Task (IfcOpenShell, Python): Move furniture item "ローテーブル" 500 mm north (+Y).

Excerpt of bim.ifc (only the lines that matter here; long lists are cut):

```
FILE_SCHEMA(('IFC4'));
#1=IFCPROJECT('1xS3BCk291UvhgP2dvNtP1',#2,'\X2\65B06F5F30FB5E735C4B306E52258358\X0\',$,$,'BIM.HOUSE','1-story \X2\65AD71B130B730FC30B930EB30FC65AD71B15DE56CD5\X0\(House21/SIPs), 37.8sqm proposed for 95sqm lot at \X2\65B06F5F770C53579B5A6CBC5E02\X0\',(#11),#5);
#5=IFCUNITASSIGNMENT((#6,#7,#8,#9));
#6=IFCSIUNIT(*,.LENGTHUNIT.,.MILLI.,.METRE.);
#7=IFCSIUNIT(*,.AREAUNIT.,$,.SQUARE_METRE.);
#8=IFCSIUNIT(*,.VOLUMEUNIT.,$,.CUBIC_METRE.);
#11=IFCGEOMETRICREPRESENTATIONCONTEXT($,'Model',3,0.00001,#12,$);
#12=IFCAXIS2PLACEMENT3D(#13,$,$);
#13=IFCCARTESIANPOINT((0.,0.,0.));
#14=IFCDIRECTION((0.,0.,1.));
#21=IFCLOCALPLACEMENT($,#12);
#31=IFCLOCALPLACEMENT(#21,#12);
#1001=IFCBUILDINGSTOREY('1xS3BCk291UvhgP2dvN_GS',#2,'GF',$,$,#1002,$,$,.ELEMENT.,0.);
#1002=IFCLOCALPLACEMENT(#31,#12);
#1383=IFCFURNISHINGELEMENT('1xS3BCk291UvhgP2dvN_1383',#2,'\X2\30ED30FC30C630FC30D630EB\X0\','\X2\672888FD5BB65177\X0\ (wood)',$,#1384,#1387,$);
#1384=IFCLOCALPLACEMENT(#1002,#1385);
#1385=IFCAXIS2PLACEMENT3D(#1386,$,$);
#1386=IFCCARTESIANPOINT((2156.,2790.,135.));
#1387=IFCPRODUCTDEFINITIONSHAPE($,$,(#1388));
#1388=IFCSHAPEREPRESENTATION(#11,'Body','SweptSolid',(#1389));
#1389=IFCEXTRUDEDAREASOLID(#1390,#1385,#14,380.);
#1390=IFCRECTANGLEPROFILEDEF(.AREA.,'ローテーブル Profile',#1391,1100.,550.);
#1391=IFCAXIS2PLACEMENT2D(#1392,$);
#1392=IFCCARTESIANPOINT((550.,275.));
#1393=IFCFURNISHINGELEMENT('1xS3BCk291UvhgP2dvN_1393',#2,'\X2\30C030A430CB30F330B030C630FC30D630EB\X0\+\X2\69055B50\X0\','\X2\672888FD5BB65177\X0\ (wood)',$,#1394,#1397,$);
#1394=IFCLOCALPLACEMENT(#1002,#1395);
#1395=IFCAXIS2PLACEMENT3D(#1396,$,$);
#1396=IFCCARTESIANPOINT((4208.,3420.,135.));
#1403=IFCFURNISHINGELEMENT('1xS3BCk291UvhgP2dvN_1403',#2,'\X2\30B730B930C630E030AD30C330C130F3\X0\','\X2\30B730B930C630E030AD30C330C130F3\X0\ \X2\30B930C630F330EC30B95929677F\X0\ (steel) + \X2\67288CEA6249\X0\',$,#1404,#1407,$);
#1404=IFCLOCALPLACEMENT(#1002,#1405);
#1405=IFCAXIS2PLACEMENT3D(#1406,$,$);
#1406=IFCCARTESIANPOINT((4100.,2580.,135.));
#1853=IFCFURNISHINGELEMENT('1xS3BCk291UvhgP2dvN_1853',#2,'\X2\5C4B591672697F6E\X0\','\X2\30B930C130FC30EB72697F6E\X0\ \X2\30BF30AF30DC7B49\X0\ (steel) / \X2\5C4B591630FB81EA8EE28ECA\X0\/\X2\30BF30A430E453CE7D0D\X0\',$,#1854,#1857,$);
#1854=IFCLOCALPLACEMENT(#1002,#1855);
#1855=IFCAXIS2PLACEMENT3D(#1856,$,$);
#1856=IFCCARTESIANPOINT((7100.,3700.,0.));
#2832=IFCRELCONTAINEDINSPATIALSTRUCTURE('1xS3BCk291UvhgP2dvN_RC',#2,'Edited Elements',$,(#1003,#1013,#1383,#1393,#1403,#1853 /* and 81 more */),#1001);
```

```python
import ifcopenshell
import ifcopenshell.api.geometry
import ifcopenshell.util.placement

model = ifcopenshell.open("bim.ifc")

item = model.by_guid("1xS3BCk291UvhgP2dvN_1383")
matrix = ifcopenshell.util.placement.get_local_placement(item.ObjectPlacement)
matrix[1, 3] += 500.0
ifcopenshell.api.geometry.edit_object_placement(model, product=item, matrix=matrix, is_si=False)

print(ifcopenshell.util.placement.get_local_placement(item.ObjectPlacement).round(3) + 0.0)

model.write("bim-out.ifc")
```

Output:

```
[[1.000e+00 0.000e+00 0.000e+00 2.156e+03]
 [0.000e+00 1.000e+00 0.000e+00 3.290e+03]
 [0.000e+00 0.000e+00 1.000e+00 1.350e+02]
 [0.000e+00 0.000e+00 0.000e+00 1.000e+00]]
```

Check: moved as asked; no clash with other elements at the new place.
